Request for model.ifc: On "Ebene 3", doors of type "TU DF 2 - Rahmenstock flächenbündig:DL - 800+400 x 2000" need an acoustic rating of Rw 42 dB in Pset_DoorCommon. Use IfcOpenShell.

First a look at what the model holds.

```python
import ifcopenshell
import ifcopenshell.util.element

model = ifcopenshell.open("model.ifc")
print(model.schema)
storey = next(s for s in model.by_type("IfcBuildingStorey") if s.Name == "Ebene 3")
doors = [e for e in ifcopenshell.util.element.get_decomposition(storey) if e.is_a("IfcDoor")]
seen = {}
for e in doors:
    element_type = ifcopenshell.util.element.get_type(e)
    key = (element_type.Name if element_type != e and element_type else None, ifcopenshell.util.element.get_pset(e, "Pset_DoorCommon", "AcousticRating"))
    seen[key] = seen.get(key, 0) + 1
for (name, value), count in sorted(seen.items(), key=str):
    print(count, "x", name, "|", value)
```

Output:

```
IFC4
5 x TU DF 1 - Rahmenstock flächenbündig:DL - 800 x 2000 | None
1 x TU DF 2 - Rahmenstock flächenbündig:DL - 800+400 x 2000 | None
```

```python
import ifcopenshell
import ifcopenshell.api.pset
import ifcopenshell.util.element

model = ifcopenshell.open("model.ifc")

storey = next(s for s in model.by_type("IfcBuildingStorey") if s.Name == "Ebene 3")
doors = [e for e in ifcopenshell.util.element.get_decomposition(storey) if e.is_a("IfcDoor")]

count = 0
for e in doors:
    element_type = ifcopenshell.util.element.get_type(e)
    if element_type in (None, e) or element_type.Name != "TU DF 2 - Rahmenstock flächenbündig:DL - 800+400 x 2000":
        continue
    # add_pset returns the element's existing set when there is one.
    pset = ifcopenshell.api.pset.add_pset(model, product=e, name="Pset_DoorCommon")
    ifcopenshell.api.pset.edit_pset(model, pset=pset, properties={"AcousticRating": "Rw 42 dB"})
    count += 1

print(count, "doors updated")

model.write("model_v2.ifc")
```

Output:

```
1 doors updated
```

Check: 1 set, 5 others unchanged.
